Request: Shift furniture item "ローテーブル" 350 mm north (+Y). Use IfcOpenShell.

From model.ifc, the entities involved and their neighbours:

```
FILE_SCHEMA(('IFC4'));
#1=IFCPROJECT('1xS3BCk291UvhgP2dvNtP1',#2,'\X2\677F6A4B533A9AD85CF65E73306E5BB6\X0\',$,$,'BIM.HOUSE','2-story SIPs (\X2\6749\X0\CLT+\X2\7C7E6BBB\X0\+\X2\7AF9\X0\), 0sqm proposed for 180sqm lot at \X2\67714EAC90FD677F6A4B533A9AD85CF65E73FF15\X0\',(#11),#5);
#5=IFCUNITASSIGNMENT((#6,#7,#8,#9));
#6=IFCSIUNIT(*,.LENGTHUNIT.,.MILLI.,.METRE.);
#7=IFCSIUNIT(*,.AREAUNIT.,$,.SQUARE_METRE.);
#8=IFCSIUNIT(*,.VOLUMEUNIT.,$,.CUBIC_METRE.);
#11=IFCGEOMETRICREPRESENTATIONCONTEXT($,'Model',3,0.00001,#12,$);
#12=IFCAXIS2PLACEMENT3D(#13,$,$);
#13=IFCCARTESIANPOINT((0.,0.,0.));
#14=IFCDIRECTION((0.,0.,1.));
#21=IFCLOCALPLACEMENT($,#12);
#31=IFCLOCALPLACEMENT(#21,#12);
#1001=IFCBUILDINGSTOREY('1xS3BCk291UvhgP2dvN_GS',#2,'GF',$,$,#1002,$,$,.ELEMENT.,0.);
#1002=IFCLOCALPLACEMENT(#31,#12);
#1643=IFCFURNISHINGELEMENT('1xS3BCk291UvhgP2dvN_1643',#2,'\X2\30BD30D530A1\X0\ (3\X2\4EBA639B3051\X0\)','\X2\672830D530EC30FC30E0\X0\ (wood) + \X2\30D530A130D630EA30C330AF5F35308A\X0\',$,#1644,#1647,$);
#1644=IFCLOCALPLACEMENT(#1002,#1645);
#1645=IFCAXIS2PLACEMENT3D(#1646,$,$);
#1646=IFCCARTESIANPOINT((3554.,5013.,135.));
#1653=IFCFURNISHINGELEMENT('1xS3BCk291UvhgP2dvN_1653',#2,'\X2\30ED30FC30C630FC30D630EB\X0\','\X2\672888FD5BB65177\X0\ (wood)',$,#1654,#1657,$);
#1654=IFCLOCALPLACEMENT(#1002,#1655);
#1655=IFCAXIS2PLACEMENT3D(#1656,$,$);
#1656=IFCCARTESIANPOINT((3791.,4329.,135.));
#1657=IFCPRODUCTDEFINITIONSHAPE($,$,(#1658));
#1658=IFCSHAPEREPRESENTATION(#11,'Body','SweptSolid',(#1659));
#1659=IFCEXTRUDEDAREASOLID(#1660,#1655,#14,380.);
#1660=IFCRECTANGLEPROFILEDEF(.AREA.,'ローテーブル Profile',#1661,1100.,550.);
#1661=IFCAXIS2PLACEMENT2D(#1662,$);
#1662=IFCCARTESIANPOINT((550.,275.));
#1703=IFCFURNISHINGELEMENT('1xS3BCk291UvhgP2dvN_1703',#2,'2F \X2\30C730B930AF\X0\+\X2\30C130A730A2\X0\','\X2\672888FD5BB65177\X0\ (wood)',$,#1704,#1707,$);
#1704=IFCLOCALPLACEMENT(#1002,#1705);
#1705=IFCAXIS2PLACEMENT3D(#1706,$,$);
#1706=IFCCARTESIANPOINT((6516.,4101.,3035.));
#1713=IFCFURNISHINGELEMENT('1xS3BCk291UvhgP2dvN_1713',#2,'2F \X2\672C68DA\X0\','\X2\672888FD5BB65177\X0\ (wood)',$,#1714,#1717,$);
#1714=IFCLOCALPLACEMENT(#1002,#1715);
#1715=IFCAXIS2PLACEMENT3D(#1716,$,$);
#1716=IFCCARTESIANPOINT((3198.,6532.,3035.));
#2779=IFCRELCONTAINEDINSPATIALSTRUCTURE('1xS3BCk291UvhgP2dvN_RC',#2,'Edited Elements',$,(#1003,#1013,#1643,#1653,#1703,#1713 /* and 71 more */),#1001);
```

```python
import ifcopenshell
import ifcopenshell.api.geometry
import ifcopenshell.util.placement
import ifcopenshell.util.unit

model = ifcopenshell.open("model.ifc")
unit_scale = ifcopenshell.util.unit.calculate_unit_scale(model)

item = model.by_guid("1xS3BCk291UvhgP2dvN_1653")
matrix = ifcopenshell.util.placement.get_local_placement(item.ObjectPlacement)
matrix[1, 3] += 0.35 / unit_scale
ifcopenshell.api.geometry.edit_object_placement(model, product=item, matrix=matrix, is_si=False)

print(ifcopenshell.util.placement.get_local_placement(item.ObjectPlacement).round(3) + 0.0)

model.write("model_updated.ifc")
```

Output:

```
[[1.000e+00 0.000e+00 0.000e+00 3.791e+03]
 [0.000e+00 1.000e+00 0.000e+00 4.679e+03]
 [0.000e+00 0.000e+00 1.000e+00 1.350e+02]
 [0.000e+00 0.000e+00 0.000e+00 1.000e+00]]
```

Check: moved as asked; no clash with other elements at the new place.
